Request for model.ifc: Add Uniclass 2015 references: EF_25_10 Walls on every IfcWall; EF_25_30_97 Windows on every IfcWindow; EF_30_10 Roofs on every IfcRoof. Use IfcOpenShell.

First a look at what the model holds.

```python
import ifcopenshell

model = ifcopenshell.open("model.ifc")
print(model.schema)
print("classifications:", [c.Name for c in model.by_type("IfcClassification")])
for ifc_class in ("IfcDoor", "IfcRoof", "IfcStair", "IfcWall", "IfcWindow"):
    print(ifc_class, len(model.by_type(ifc_class)))
```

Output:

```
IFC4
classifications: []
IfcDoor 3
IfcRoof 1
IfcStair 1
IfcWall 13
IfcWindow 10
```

```python
import ifcopenshell
import ifcopenshell.api.classification

model = ifcopenshell.open("model.ifc")

system = ifcopenshell.api.classification.add_classification(model, classification="Uniclass 2015")

codes = {
    "IfcWall": ("EF_25_10", "Walls"),
    "IfcWindow": ("EF_25_30_97", "Windows"),
    "IfcRoof": ("EF_30_10", "Roofs"),
}
for ifc_class, (code, name) in codes.items():
    products = model.by_type(ifc_class)
    ifcopenshell.api.classification.add_reference(
        model, products=products, classification=system, identification=code, name=name
    )
    print(code, len(products))

model.write("model_edited.ifc")
```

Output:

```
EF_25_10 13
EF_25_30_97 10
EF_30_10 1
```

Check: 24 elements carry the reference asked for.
